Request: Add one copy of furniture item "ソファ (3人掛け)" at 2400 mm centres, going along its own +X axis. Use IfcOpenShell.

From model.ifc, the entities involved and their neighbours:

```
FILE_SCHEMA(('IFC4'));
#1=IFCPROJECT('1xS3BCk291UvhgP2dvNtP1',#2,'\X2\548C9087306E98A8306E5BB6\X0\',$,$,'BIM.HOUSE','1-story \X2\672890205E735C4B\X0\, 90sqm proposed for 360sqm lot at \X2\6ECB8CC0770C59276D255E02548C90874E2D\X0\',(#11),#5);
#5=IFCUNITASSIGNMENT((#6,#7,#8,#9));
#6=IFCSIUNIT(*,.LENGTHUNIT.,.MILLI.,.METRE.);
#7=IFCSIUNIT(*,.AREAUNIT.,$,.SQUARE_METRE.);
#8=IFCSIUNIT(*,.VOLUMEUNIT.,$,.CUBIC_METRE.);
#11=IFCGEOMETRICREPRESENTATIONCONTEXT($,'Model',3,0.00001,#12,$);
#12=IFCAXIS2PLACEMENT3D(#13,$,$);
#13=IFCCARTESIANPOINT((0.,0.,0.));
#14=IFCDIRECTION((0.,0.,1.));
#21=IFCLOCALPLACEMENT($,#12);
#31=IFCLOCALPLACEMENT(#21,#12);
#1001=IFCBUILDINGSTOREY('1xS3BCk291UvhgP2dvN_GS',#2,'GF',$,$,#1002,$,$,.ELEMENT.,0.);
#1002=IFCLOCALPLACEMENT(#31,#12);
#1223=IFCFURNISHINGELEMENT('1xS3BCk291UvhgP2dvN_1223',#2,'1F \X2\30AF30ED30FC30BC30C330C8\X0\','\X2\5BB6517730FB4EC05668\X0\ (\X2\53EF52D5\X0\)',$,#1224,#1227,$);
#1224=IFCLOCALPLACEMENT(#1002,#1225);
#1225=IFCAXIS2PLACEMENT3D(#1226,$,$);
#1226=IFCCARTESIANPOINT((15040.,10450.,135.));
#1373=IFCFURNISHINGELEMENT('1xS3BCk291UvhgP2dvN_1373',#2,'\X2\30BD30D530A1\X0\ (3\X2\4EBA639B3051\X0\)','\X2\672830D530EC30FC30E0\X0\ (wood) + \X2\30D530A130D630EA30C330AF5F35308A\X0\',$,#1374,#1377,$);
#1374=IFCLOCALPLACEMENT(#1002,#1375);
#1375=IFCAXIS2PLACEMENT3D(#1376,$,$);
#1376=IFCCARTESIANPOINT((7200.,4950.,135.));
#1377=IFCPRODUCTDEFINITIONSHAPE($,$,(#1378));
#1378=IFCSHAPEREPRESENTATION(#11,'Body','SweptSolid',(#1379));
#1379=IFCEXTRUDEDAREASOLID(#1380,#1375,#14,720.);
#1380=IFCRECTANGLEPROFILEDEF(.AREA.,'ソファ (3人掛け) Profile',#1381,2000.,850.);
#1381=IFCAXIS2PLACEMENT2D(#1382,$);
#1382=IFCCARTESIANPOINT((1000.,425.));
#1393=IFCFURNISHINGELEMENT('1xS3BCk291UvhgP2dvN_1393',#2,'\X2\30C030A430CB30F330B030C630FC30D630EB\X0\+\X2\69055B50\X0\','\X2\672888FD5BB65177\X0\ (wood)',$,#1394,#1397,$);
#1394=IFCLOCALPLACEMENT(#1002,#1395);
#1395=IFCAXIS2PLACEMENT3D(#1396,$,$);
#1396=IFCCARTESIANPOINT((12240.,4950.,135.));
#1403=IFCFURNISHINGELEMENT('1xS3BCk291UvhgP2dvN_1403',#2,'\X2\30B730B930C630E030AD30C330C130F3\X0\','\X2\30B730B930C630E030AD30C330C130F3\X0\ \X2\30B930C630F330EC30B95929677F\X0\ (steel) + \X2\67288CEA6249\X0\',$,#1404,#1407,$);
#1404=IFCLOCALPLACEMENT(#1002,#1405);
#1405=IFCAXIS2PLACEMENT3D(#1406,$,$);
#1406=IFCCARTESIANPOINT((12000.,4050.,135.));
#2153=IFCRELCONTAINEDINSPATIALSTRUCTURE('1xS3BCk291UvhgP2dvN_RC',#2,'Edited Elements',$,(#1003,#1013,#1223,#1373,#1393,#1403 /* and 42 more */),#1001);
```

```python
import ifcopenshell
import ifcopenshell.api.geometry
import ifcopenshell.api.root
import ifcopenshell.util.element
import ifcopenshell.util.placement

model = ifcopenshell.open("model.ifc")


def reuse_history(source, copy):
    """copy_class also copies each property set's owner history, people and application; keep the originals."""
    for rel in copy.IsDefinedBy:
        if rel.is_a("IfcRelDefinesByProperties") and (history := rel.RelatingPropertyDefinition.OwnerHistory):
            rel.RelatingPropertyDefinition.OwnerHistory = source.OwnerHistory
            ifcopenshell.util.element.remove_deep2(model, history)


source = model.by_guid("1xS3BCk291UvhgP2dvN_1373")
base = ifcopenshell.util.placement.get_local_placement(source.ObjectPlacement)
step = base[:3, 0] * 2400.0

for i in range(1, 2):
    copy = ifcopenshell.api.root.copy_class(model, product=source)
    copy.Representation = ifcopenshell.util.element.copy_deep(
        model, source.Representation, exclude=["IfcGeometricRepresentationContext", "IfcRepresentationMap"]
    )
    reuse_history(source, copy)
    matrix = base.copy()
    matrix[:3, 3] += i * step
    print("added at", matrix[:3, 3].round(3) + 0.0)
    ifcopenshell.api.geometry.edit_object_placement(model, product=copy, matrix=matrix, is_si=False)

model.write("model_updated.ifc")
```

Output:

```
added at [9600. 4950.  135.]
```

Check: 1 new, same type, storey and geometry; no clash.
